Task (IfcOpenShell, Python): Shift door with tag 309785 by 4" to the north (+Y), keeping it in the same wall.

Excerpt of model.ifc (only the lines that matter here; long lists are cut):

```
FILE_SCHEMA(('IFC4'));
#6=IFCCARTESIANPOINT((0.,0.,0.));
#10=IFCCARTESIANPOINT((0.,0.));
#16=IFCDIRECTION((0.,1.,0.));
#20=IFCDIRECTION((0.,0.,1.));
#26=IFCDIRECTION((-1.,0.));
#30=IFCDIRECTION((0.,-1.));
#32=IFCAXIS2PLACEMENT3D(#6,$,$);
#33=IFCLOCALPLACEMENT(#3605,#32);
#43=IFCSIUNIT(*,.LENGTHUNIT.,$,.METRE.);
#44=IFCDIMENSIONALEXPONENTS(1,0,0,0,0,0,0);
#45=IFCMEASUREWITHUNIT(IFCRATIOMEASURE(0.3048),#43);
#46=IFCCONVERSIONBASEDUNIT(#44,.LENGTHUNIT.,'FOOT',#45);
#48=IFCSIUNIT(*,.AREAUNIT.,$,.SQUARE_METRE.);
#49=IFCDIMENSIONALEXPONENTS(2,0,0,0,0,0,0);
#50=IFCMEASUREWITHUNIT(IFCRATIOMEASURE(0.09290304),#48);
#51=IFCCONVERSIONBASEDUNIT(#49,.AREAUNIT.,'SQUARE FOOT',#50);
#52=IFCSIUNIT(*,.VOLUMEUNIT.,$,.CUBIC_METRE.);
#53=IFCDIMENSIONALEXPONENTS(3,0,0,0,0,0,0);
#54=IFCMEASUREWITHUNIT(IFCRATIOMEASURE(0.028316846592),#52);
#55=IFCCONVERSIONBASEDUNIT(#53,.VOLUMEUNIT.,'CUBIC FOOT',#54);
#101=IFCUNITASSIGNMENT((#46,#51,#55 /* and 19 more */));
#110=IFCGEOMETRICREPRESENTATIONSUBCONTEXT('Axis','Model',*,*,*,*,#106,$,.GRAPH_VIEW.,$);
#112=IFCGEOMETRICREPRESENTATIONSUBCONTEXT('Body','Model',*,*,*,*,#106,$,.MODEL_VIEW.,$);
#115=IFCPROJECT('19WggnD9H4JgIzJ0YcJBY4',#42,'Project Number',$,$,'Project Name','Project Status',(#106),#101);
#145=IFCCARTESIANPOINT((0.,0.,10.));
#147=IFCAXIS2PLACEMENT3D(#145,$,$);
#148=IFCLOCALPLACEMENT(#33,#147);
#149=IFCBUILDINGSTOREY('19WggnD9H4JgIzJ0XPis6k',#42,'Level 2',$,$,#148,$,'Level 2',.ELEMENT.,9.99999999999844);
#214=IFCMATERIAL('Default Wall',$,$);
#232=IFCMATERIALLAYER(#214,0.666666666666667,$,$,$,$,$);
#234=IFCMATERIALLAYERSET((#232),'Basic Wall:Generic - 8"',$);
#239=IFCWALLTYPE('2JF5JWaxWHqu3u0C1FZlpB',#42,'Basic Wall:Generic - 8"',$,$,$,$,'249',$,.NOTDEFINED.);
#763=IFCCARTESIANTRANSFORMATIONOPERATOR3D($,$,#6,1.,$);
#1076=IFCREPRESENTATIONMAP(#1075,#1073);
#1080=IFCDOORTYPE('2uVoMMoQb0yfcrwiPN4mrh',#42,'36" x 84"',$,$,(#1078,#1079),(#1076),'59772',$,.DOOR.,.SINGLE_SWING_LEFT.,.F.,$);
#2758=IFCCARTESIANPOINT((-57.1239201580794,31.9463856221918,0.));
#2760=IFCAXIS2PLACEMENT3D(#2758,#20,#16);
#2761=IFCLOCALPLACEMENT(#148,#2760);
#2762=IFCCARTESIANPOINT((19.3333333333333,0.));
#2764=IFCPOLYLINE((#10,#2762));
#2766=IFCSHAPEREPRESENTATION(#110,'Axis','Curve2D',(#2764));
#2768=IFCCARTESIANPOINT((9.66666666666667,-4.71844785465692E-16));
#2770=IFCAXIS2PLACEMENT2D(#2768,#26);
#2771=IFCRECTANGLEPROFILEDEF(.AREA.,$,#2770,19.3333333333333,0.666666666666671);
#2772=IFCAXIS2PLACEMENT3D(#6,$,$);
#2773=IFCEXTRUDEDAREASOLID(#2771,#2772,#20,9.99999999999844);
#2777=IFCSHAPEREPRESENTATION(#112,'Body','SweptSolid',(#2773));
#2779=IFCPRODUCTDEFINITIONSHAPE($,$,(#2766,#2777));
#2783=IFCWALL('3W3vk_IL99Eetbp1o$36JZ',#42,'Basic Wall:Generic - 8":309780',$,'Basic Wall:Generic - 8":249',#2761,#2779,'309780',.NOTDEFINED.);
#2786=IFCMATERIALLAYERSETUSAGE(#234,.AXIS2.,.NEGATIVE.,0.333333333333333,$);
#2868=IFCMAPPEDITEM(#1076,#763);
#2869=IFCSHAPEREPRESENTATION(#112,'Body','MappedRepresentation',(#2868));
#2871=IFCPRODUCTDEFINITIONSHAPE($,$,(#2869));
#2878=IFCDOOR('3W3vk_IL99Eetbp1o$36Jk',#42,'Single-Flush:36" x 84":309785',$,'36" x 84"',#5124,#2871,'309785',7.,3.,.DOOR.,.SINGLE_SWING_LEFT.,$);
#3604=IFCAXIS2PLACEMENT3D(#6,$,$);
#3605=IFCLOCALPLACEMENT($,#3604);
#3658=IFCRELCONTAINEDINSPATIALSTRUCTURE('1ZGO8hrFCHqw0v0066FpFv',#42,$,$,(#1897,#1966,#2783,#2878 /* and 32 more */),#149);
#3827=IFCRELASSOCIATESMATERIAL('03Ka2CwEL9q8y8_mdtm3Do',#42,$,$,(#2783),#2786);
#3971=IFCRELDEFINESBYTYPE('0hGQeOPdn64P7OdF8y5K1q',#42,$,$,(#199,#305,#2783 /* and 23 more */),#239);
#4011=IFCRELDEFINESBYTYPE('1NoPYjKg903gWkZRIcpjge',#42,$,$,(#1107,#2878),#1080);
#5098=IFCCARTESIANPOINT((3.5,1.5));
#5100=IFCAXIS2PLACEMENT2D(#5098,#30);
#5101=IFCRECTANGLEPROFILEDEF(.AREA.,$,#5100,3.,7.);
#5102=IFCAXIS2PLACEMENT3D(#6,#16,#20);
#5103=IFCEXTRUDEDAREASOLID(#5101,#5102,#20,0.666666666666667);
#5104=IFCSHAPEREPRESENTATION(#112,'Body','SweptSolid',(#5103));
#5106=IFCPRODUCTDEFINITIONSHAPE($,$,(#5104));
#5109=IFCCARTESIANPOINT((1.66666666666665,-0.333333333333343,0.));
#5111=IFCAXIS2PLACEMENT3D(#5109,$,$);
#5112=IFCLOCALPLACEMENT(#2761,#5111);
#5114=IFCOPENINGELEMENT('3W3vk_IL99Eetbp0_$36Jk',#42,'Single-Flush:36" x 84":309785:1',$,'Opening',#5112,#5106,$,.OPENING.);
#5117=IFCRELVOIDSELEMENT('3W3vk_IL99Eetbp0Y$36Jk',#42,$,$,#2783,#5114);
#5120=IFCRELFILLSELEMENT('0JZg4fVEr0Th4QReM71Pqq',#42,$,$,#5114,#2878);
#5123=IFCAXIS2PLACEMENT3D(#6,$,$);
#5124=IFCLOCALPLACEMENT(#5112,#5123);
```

```python
import ifcopenshell
import ifcopenshell.api.geometry
import ifcopenshell.util.placement
import ifcopenshell.util.unit

model = ifcopenshell.open("model.ifc")
unit_scale = ifcopenshell.util.unit.calculate_unit_scale(model)

door = model.by_id(2878)
opening = door.FillsVoids[0].RelatingOpeningElement
wall = opening.VoidsElements[0].RelatingBuildingElement

wall_matrix = ifcopenshell.util.placement.get_local_placement(wall.ObjectPlacement)
shift = wall_matrix[:3, 0] * 4 * 0.0254 / unit_scale
before = ifcopenshell.util.placement.get_local_placement(door.ObjectPlacement)[:3, 3].copy()

# The door is placed relative to its opening, so it follows when the opening moves.
matrix = ifcopenshell.util.placement.get_local_placement(opening.ObjectPlacement)
matrix[:3, 3] += shift
ifcopenshell.api.geometry.edit_object_placement(
    model, product=opening, matrix=matrix, is_si=False, should_transform_children=True
)

after = ifcopenshell.util.placement.get_local_placement(door.ObjectPlacement)[:3, 3]
print("door moved by", (after - before).round(3) + 0.0)

model.write("model_updated.ifc")
```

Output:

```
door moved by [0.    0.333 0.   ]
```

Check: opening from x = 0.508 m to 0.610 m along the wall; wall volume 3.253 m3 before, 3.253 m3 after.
